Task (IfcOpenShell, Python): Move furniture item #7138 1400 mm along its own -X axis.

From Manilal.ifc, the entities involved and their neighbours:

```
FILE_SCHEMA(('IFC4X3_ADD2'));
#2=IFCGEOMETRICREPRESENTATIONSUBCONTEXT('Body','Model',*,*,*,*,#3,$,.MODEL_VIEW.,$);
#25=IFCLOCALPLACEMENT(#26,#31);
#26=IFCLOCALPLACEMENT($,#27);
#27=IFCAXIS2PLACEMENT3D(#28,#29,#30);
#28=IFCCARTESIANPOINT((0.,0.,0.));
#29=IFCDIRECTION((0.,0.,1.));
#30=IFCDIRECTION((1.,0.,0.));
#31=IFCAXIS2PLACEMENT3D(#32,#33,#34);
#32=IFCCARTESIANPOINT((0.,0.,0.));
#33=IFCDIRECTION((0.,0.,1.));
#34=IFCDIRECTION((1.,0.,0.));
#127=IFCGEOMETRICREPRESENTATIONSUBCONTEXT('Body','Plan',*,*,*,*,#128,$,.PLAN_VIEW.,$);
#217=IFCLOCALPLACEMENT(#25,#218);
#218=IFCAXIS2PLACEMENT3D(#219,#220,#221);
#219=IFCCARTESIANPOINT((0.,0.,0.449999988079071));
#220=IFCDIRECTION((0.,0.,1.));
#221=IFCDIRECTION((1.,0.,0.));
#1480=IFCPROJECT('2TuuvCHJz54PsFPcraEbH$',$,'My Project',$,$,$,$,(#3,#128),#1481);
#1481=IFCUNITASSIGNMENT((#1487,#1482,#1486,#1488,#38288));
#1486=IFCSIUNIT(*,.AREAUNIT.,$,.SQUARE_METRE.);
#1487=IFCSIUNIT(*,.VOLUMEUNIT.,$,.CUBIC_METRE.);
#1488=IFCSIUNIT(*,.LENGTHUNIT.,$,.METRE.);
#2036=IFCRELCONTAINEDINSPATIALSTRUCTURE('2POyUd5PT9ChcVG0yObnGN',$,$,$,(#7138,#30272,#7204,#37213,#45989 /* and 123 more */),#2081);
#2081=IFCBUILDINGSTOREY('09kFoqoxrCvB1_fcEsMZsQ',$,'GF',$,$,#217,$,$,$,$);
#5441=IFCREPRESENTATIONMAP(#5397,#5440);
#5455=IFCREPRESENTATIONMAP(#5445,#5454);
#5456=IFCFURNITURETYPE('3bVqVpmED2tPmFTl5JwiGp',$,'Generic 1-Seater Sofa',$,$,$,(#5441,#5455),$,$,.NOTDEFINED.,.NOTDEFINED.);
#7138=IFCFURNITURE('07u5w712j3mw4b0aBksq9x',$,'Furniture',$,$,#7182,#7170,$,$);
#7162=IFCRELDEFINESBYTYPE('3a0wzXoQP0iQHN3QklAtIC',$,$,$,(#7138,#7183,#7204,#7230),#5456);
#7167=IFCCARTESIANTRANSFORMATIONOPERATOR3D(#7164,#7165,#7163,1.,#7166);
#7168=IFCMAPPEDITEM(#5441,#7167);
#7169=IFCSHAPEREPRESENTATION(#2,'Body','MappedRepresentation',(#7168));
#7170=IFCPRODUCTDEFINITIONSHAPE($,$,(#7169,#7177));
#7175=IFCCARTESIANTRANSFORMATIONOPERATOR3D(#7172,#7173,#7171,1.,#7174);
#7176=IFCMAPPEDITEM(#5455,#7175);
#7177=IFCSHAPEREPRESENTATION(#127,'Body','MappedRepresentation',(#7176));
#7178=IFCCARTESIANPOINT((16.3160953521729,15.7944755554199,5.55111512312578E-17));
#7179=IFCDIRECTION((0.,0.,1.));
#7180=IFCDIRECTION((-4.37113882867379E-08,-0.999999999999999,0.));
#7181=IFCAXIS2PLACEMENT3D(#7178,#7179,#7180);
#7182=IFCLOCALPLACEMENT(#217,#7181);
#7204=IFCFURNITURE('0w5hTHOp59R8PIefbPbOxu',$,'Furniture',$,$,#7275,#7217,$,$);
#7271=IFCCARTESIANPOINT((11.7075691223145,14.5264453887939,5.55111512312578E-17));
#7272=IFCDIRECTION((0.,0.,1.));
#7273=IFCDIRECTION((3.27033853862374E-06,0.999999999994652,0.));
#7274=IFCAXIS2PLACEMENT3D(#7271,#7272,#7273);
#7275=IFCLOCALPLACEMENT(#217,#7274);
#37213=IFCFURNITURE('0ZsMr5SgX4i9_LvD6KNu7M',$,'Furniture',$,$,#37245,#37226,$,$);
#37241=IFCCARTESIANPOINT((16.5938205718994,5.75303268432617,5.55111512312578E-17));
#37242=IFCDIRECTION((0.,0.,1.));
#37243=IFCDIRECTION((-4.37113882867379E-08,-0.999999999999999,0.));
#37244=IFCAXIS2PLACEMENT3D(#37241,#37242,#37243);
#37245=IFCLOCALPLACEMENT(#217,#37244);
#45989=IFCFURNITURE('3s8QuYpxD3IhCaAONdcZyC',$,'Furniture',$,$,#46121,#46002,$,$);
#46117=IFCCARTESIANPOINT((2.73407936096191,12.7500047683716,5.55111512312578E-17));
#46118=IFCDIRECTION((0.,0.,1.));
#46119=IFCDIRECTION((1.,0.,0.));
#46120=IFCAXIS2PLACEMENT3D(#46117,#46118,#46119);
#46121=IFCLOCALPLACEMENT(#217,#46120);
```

```python
import ifcopenshell
import ifcopenshell.api.geometry
import ifcopenshell.util.placement
import ifcopenshell.util.unit

model = ifcopenshell.open("Manilal.ifc")
unit_scale = ifcopenshell.util.unit.calculate_unit_scale(model)

item = model.by_guid("07u5w712j3mw4b0aBksq9x")
matrix = ifcopenshell.util.placement.get_local_placement(item.ObjectPlacement)
matrix[:3, 3] -= matrix[:3, 0] * 1.4 / unit_scale
ifcopenshell.api.geometry.edit_object_placement(model, product=item, matrix=matrix, is_si=False)

print(ifcopenshell.util.placement.get_local_placement(item.ObjectPlacement).round(3) + 0.0)

model.write("Manilal_updated.ifc")
```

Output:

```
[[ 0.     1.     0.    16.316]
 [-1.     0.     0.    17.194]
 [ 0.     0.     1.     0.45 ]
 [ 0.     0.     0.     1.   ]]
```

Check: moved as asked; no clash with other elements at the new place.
